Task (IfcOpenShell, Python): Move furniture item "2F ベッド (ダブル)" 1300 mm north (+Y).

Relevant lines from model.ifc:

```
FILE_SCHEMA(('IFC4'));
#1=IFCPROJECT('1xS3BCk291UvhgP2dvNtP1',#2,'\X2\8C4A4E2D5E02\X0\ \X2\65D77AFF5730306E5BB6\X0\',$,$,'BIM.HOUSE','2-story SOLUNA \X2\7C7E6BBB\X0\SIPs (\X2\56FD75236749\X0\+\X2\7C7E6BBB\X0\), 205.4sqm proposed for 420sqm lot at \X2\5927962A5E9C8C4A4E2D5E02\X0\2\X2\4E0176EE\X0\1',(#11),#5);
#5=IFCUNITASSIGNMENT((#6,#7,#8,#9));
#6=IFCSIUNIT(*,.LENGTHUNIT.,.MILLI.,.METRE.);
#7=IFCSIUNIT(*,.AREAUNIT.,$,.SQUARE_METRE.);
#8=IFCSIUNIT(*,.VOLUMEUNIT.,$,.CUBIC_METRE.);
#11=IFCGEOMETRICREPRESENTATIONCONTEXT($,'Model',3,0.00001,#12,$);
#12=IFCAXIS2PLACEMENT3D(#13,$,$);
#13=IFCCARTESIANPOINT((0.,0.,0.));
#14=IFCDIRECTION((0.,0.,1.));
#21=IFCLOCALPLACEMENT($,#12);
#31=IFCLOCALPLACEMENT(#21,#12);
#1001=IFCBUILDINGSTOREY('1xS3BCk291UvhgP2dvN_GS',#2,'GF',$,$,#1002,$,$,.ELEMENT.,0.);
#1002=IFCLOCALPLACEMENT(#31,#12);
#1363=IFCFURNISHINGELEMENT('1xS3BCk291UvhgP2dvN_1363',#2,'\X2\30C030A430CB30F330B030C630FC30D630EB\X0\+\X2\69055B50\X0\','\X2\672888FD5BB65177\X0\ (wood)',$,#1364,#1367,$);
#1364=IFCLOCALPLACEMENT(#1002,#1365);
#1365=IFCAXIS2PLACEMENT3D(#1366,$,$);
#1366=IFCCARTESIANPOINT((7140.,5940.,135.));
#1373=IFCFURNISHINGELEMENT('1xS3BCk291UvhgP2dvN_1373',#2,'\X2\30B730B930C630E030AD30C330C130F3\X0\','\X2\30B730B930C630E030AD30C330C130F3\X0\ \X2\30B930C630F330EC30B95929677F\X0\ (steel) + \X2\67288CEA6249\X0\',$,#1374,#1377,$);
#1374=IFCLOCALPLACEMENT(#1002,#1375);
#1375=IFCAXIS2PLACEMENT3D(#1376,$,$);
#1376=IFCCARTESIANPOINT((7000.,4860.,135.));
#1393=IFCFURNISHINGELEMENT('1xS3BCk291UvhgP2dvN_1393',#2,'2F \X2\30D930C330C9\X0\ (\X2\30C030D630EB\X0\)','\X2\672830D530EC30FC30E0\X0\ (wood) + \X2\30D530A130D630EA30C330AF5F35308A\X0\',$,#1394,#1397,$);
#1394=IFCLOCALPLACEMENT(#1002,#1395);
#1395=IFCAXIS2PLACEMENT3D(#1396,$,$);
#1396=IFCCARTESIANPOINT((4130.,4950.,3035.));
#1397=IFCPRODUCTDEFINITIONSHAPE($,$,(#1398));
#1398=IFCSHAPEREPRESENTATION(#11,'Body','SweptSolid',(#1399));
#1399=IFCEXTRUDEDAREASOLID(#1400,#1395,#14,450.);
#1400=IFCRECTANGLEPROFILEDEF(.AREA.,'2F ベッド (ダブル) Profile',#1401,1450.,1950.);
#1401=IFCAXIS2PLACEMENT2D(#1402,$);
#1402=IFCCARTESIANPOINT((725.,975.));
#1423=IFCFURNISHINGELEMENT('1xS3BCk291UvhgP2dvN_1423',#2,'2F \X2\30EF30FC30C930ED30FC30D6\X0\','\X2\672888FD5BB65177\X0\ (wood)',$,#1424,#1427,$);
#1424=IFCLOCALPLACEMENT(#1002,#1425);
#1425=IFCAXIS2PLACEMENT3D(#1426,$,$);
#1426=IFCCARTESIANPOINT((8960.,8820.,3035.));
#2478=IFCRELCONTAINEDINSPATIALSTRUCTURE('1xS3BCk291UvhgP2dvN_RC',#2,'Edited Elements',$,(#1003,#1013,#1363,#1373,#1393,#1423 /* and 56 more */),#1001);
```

```python
import ifcopenshell
import ifcopenshell.api.geometry
import ifcopenshell.util.placement
import ifcopenshell.util.unit

model = ifcopenshell.open("model.ifc")
unit_scale = ifcopenshell.util.unit.calculate_unit_scale(model)

item = model.by_guid("1xS3BCk291UvhgP2dvN_1393")
matrix = ifcopenshell.util.placement.get_local_placement(item.ObjectPlacement)
matrix[1, 3] += 1.3 / unit_scale
ifcopenshell.api.geometry.edit_object_placement(model, product=item, matrix=matrix, is_si=False)

print(ifcopenshell.util.placement.get_local_placement(item.ObjectPlacement).round(3) + 0.0)

model.write("model_updated.ifc")
```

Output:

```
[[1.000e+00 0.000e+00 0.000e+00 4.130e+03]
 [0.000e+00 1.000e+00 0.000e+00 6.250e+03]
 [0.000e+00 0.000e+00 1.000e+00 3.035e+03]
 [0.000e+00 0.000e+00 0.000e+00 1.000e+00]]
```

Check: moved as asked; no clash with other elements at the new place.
